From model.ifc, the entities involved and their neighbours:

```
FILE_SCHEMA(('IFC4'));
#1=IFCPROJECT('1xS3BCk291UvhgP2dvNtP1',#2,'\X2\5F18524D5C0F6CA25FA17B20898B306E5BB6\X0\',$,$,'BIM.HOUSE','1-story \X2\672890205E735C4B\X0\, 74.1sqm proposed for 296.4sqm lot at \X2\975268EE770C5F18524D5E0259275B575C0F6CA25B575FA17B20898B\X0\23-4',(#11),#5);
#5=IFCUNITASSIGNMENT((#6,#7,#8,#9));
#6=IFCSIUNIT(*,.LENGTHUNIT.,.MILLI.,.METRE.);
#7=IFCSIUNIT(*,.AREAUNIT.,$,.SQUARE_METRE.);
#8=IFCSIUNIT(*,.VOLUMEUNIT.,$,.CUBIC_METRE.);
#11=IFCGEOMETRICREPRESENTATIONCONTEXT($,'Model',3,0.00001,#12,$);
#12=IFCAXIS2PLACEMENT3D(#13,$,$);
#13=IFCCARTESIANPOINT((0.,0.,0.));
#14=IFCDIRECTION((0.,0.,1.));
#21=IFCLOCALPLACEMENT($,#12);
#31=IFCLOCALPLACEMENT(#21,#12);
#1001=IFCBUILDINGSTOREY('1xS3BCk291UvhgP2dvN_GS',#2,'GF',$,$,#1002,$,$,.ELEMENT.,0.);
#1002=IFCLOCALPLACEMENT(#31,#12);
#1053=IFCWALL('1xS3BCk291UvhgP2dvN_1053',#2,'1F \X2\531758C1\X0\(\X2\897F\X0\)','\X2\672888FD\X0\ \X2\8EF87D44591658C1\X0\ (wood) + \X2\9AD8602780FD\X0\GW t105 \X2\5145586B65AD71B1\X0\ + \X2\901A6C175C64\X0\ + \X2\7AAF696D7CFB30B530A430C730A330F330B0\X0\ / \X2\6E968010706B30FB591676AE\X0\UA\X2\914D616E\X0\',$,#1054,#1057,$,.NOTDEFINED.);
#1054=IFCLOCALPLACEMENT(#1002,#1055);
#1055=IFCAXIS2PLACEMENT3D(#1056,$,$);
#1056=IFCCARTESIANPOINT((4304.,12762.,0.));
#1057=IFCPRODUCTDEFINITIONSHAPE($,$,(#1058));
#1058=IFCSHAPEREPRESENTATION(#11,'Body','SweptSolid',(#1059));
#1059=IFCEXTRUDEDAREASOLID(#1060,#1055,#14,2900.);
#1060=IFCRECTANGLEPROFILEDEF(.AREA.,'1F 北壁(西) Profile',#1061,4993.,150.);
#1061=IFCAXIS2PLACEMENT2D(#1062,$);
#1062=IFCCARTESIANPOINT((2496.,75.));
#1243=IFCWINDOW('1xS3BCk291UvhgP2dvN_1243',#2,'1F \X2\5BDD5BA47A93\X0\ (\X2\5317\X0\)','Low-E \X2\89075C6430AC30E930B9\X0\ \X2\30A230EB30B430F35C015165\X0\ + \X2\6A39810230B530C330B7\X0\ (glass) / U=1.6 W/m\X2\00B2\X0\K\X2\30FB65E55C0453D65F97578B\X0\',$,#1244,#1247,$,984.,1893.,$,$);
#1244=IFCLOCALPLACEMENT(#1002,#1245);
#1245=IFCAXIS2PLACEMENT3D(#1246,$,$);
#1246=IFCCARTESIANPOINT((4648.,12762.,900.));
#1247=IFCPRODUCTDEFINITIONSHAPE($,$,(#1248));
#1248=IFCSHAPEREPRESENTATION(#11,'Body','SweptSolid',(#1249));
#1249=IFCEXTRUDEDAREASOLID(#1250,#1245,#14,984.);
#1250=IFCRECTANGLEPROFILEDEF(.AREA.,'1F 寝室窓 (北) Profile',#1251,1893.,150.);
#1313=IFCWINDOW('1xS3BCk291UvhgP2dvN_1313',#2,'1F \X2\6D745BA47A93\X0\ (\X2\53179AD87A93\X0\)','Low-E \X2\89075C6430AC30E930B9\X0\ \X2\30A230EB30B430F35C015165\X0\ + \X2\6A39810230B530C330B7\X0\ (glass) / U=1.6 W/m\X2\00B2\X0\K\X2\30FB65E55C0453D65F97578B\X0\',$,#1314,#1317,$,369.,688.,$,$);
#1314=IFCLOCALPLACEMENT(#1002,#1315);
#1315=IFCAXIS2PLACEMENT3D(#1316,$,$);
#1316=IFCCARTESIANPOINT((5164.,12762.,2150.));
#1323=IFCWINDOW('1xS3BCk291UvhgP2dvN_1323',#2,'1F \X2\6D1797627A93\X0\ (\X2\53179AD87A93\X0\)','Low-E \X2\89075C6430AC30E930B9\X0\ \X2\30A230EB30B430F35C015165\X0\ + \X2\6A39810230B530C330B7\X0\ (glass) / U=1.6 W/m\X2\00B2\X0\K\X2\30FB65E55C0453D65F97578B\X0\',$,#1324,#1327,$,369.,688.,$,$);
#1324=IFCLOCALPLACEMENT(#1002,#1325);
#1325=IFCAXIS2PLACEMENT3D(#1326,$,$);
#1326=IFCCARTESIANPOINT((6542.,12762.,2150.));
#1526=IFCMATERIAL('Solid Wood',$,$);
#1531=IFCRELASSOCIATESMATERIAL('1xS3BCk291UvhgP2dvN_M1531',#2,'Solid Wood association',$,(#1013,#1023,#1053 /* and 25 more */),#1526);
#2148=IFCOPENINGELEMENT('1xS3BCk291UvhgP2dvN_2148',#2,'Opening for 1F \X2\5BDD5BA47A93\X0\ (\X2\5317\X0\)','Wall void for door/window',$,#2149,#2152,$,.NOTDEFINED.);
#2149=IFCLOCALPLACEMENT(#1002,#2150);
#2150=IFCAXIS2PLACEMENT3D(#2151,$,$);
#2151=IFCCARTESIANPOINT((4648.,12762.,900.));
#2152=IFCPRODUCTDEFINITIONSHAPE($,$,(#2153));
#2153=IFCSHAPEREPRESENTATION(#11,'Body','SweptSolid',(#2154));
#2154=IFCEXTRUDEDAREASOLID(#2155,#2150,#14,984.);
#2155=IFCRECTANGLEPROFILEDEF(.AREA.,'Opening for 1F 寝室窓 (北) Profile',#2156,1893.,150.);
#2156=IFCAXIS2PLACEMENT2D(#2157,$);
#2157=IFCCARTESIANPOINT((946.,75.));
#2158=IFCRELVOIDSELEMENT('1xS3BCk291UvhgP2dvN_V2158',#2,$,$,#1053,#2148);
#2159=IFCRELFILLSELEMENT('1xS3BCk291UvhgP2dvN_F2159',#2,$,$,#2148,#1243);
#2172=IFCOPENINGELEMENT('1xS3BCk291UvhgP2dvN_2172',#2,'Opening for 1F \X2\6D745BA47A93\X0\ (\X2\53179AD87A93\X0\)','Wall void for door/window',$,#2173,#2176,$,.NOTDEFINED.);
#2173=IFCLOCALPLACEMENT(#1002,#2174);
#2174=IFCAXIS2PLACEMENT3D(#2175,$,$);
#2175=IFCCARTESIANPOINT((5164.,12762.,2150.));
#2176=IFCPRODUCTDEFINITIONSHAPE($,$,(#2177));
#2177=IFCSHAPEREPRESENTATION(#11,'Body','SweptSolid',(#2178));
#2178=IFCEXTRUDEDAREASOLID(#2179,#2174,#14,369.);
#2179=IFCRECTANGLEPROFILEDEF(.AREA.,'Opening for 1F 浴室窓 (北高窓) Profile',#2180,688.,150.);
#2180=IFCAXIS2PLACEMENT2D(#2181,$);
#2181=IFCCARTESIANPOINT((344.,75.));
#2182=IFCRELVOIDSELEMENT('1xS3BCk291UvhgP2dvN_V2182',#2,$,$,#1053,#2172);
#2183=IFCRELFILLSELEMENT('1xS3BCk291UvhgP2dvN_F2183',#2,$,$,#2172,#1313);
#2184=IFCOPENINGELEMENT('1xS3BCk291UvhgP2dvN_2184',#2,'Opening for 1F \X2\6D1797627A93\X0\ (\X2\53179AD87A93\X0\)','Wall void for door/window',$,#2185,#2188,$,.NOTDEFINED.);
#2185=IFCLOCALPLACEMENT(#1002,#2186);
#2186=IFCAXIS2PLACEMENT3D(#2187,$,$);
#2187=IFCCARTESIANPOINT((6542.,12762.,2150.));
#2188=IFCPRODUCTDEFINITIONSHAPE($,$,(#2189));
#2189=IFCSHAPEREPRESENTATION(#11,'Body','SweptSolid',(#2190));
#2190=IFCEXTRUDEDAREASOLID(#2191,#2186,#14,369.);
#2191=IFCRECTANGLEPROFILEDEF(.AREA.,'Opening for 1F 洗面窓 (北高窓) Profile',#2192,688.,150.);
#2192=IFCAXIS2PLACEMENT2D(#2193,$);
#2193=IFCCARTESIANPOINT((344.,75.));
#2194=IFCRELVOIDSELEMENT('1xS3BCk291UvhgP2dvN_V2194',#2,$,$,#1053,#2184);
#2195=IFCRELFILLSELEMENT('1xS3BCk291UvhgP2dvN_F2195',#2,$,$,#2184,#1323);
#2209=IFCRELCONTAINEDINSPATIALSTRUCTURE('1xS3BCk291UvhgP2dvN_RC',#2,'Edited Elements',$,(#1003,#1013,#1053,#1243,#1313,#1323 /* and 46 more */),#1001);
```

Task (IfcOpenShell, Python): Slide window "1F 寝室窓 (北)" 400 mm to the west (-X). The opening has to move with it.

```python
import ifcopenshell
import ifcopenshell.api.geometry
import ifcopenshell.util.placement
import ifcopenshell.util.unit

model = ifcopenshell.open("model.ifc")
unit_scale = ifcopenshell.util.unit.calculate_unit_scale(model)

window = model.by_id(1243)
opening = window.FillsVoids[0].RelatingOpeningElement
wall = opening.VoidsElements[0].RelatingBuildingElement

wall_matrix = ifcopenshell.util.placement.get_local_placement(wall.ObjectPlacement)
shift = wall_matrix[:3, 0] * -0.4 / unit_scale
before = ifcopenshell.util.placement.get_local_placement(window.ObjectPlacement)[:3, 3].copy()

# The window is not placed relative to its opening, so move both.
for product in (opening, window):
    matrix = ifcopenshell.util.placement.get_local_placement(product.ObjectPlacement)
    matrix[:3, 3] += shift
    ifcopenshell.api.geometry.edit_object_placement(model, product=product, matrix=matrix, is_si=False)

after = ifcopenshell.util.placement.get_local_placement(window.ObjectPlacement)[:3, 3]
print("window moved by", (after - before).round(3) + 0.0)

model.write("model-out.ifc")
```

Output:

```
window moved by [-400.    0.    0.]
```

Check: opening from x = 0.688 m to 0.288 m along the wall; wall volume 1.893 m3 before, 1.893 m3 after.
